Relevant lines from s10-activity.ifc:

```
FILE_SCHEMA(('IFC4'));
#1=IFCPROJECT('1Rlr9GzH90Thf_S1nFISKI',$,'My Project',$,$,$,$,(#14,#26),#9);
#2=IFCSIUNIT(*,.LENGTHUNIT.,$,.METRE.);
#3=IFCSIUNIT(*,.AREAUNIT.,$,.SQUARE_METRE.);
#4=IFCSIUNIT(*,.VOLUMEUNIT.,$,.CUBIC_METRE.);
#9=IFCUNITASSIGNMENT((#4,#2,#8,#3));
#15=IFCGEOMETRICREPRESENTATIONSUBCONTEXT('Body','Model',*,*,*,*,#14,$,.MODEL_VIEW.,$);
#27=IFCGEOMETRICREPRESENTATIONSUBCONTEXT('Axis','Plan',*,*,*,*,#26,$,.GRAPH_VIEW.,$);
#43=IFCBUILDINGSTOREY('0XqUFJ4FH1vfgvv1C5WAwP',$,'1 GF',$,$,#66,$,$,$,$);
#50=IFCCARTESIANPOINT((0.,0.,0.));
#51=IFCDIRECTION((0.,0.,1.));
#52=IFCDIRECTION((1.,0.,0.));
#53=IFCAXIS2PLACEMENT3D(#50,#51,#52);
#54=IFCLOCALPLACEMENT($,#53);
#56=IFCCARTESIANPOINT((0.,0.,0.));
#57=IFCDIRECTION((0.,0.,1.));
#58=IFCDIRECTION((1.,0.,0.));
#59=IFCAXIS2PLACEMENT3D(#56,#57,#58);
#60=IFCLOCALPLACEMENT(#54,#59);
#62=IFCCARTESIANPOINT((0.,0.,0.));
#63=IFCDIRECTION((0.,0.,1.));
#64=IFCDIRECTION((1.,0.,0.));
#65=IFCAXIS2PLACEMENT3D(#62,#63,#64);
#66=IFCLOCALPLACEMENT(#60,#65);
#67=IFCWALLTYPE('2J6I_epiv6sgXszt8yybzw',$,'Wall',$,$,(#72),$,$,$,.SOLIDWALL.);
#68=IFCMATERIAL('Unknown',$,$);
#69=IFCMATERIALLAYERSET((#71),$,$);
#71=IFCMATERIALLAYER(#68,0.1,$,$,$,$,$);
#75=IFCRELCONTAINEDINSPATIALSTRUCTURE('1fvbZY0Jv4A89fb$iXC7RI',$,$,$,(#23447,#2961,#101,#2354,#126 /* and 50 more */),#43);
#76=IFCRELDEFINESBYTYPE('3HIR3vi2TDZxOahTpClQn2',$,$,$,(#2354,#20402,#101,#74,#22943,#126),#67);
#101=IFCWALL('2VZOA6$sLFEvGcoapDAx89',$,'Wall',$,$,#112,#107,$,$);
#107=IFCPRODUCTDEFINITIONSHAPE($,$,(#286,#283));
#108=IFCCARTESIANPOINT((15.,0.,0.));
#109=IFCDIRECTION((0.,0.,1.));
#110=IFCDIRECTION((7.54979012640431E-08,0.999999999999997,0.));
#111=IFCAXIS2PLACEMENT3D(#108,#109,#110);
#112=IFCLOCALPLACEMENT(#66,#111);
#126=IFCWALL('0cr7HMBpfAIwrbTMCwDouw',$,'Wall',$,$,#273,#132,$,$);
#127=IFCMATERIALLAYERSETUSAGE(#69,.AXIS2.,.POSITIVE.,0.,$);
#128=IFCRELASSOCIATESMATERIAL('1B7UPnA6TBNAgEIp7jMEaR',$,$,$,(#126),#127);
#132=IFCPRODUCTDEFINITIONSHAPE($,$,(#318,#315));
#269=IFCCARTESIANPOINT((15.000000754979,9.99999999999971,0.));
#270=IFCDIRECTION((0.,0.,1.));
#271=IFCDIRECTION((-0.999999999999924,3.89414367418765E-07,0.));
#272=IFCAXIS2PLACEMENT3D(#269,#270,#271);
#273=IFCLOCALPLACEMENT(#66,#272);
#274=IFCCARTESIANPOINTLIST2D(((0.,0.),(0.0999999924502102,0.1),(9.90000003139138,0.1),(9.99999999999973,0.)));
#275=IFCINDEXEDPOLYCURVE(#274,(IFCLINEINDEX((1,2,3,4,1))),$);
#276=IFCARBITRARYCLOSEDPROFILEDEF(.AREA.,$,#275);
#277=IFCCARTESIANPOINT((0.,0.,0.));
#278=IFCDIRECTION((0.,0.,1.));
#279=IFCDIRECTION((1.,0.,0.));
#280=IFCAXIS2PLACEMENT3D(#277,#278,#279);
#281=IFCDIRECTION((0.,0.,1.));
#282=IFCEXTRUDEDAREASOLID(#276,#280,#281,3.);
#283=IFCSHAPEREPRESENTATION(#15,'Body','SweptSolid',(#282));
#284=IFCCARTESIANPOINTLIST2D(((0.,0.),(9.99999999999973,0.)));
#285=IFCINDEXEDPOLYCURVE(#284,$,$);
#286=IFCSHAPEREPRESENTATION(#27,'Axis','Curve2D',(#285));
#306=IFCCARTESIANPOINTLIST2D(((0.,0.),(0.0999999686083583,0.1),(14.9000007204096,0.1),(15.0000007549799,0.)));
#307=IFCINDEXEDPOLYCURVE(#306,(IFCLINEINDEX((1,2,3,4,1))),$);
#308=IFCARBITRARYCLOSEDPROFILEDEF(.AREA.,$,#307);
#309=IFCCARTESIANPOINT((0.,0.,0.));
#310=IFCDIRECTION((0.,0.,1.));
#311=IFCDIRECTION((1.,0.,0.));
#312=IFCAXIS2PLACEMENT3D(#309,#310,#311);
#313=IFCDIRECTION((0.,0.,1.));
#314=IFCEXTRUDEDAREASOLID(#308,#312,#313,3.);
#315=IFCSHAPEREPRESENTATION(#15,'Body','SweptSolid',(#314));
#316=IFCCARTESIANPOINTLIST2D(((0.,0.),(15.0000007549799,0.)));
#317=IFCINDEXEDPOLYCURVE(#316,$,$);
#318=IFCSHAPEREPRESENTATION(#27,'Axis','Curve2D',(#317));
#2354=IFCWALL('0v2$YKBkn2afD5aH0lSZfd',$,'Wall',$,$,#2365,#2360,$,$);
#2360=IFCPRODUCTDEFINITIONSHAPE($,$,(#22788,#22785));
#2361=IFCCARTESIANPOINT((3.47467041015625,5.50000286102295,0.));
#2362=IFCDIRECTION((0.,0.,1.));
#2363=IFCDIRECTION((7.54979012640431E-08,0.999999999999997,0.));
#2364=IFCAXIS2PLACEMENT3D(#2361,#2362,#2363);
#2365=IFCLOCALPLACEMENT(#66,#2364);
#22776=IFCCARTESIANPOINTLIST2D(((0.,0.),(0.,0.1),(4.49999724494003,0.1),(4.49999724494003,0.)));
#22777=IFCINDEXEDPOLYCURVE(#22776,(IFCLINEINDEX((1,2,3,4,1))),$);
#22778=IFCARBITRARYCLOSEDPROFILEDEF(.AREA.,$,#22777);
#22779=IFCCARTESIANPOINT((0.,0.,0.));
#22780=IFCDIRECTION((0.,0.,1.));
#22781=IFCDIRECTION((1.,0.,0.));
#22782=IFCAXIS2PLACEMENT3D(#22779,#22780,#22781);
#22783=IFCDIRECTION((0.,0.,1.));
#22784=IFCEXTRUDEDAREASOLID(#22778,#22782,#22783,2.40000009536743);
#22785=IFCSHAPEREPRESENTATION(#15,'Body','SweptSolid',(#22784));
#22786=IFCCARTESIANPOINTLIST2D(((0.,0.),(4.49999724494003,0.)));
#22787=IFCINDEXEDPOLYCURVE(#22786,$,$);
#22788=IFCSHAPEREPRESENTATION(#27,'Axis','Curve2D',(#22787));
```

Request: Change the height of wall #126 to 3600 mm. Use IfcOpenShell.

```python
import ifcopenshell
import ifcopenshell.geom
import ifcopenshell.util.representation
import ifcopenshell.util.shape

model = ifcopenshell.open("s10-activity.ifc")
settings = ifcopenshell.geom.settings()


def volume(element):
    """Net volume in cubic metres, openings subtracted."""
    shape = ifcopenshell.geom.create_shape(settings, element)
    return ifcopenshell.util.shape.get_volume(shape.geometry)


wall = model.by_id(126)
before = volume(wall)

body = ifcopenshell.util.representation.get_representation(wall, "Model", "Body")
solid = body.Items[0]
old_height = solid.Depth
solid.Depth = 3.6
after = volume(wall)

print(f"height {old_height:g} -> {solid.Depth:g}, volume {before:.3f} -> {after:.3f} m3")

model.write("s10-activity_updated.ifc")
```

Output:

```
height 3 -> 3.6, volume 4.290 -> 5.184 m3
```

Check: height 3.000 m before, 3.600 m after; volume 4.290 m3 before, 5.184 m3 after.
